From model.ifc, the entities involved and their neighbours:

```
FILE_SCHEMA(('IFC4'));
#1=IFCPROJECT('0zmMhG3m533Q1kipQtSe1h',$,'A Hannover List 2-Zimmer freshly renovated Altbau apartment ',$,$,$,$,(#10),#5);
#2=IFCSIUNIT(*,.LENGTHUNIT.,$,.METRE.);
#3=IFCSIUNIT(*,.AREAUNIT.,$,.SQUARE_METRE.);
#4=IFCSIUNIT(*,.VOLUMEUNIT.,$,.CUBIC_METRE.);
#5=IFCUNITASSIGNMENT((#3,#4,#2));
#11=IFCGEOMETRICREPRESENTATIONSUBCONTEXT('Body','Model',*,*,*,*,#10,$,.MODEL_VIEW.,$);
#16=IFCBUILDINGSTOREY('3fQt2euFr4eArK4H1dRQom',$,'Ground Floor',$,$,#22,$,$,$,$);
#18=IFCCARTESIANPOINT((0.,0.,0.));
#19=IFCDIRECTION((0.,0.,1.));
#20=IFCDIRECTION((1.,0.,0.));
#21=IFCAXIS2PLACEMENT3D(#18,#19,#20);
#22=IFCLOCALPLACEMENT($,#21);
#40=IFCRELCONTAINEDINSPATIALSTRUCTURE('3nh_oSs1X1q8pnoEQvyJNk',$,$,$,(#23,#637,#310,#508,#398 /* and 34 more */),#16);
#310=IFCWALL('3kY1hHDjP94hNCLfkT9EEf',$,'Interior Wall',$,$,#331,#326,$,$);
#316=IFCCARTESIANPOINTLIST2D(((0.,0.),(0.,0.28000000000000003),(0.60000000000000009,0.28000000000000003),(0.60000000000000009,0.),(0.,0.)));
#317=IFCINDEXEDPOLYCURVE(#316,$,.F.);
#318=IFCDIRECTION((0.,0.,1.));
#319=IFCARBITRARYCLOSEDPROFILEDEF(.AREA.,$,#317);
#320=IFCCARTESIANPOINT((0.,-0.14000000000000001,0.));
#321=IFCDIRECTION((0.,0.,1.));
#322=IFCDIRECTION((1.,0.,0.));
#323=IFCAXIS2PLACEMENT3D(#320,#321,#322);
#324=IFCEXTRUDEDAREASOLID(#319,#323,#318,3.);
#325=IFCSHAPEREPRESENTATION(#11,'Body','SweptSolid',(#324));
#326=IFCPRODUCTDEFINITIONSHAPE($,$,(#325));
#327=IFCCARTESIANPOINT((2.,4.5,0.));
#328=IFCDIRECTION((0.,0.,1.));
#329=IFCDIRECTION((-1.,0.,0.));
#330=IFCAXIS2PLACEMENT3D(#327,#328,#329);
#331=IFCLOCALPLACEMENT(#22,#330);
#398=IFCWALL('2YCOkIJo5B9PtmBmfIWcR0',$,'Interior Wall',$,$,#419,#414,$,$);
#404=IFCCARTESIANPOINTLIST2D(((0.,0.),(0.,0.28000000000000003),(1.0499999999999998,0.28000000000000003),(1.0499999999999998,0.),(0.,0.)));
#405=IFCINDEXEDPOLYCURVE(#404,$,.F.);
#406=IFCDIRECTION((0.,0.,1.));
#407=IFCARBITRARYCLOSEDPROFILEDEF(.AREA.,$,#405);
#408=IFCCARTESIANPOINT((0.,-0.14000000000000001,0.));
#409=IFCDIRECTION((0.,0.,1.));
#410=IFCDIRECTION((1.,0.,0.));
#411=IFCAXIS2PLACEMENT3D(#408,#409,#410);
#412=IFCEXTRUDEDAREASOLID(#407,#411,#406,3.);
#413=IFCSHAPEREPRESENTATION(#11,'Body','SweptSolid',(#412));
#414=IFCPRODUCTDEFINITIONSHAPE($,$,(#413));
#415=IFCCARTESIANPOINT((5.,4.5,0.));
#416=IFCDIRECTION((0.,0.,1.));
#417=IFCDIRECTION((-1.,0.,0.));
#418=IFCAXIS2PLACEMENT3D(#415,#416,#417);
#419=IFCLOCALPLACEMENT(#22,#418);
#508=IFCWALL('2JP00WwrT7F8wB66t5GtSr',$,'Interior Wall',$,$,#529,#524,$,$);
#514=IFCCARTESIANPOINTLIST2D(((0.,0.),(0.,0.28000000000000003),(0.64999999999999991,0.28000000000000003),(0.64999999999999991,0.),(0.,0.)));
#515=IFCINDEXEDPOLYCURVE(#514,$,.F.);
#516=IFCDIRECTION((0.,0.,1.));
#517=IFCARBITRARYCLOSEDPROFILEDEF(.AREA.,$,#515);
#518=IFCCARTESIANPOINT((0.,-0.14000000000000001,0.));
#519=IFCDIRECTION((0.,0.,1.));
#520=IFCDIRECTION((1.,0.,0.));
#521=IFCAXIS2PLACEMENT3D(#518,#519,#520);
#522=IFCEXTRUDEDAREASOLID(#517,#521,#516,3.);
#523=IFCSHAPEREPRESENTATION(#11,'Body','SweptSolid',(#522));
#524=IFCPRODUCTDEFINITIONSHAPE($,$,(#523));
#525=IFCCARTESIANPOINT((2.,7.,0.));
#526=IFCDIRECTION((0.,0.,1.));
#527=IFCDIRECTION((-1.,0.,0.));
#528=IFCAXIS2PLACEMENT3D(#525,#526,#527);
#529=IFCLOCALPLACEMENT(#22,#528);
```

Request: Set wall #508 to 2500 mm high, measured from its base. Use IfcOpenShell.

```python
import ifcopenshell
import ifcopenshell.geom
import ifcopenshell.util.representation
import ifcopenshell.util.shape
import ifcopenshell.util.unit

model = ifcopenshell.open("model.ifc")
unit_scale = ifcopenshell.util.unit.calculate_unit_scale(model)
settings = ifcopenshell.geom.settings()


def volume(element):
    """Net volume in cubic metres, openings subtracted."""
    shape = ifcopenshell.geom.create_shape(settings, element)
    return ifcopenshell.util.shape.get_volume(shape.geometry)


wall = model.by_guid("2JP00WwrT7F8wB66t5GtSr")
before = volume(wall)

body = ifcopenshell.util.representation.get_representation(wall, "Model", "Body")
solid = body.Items[0]
old_height = solid.Depth
solid.Depth = 2.5 / unit_scale
after = volume(wall)

print(f"height {old_height:g} -> {solid.Depth:g}, volume {before:.3f} -> {after:.3f} m3")

model.write("model-out.ifc")
```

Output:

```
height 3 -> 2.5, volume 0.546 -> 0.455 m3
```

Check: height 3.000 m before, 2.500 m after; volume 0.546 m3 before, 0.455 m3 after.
